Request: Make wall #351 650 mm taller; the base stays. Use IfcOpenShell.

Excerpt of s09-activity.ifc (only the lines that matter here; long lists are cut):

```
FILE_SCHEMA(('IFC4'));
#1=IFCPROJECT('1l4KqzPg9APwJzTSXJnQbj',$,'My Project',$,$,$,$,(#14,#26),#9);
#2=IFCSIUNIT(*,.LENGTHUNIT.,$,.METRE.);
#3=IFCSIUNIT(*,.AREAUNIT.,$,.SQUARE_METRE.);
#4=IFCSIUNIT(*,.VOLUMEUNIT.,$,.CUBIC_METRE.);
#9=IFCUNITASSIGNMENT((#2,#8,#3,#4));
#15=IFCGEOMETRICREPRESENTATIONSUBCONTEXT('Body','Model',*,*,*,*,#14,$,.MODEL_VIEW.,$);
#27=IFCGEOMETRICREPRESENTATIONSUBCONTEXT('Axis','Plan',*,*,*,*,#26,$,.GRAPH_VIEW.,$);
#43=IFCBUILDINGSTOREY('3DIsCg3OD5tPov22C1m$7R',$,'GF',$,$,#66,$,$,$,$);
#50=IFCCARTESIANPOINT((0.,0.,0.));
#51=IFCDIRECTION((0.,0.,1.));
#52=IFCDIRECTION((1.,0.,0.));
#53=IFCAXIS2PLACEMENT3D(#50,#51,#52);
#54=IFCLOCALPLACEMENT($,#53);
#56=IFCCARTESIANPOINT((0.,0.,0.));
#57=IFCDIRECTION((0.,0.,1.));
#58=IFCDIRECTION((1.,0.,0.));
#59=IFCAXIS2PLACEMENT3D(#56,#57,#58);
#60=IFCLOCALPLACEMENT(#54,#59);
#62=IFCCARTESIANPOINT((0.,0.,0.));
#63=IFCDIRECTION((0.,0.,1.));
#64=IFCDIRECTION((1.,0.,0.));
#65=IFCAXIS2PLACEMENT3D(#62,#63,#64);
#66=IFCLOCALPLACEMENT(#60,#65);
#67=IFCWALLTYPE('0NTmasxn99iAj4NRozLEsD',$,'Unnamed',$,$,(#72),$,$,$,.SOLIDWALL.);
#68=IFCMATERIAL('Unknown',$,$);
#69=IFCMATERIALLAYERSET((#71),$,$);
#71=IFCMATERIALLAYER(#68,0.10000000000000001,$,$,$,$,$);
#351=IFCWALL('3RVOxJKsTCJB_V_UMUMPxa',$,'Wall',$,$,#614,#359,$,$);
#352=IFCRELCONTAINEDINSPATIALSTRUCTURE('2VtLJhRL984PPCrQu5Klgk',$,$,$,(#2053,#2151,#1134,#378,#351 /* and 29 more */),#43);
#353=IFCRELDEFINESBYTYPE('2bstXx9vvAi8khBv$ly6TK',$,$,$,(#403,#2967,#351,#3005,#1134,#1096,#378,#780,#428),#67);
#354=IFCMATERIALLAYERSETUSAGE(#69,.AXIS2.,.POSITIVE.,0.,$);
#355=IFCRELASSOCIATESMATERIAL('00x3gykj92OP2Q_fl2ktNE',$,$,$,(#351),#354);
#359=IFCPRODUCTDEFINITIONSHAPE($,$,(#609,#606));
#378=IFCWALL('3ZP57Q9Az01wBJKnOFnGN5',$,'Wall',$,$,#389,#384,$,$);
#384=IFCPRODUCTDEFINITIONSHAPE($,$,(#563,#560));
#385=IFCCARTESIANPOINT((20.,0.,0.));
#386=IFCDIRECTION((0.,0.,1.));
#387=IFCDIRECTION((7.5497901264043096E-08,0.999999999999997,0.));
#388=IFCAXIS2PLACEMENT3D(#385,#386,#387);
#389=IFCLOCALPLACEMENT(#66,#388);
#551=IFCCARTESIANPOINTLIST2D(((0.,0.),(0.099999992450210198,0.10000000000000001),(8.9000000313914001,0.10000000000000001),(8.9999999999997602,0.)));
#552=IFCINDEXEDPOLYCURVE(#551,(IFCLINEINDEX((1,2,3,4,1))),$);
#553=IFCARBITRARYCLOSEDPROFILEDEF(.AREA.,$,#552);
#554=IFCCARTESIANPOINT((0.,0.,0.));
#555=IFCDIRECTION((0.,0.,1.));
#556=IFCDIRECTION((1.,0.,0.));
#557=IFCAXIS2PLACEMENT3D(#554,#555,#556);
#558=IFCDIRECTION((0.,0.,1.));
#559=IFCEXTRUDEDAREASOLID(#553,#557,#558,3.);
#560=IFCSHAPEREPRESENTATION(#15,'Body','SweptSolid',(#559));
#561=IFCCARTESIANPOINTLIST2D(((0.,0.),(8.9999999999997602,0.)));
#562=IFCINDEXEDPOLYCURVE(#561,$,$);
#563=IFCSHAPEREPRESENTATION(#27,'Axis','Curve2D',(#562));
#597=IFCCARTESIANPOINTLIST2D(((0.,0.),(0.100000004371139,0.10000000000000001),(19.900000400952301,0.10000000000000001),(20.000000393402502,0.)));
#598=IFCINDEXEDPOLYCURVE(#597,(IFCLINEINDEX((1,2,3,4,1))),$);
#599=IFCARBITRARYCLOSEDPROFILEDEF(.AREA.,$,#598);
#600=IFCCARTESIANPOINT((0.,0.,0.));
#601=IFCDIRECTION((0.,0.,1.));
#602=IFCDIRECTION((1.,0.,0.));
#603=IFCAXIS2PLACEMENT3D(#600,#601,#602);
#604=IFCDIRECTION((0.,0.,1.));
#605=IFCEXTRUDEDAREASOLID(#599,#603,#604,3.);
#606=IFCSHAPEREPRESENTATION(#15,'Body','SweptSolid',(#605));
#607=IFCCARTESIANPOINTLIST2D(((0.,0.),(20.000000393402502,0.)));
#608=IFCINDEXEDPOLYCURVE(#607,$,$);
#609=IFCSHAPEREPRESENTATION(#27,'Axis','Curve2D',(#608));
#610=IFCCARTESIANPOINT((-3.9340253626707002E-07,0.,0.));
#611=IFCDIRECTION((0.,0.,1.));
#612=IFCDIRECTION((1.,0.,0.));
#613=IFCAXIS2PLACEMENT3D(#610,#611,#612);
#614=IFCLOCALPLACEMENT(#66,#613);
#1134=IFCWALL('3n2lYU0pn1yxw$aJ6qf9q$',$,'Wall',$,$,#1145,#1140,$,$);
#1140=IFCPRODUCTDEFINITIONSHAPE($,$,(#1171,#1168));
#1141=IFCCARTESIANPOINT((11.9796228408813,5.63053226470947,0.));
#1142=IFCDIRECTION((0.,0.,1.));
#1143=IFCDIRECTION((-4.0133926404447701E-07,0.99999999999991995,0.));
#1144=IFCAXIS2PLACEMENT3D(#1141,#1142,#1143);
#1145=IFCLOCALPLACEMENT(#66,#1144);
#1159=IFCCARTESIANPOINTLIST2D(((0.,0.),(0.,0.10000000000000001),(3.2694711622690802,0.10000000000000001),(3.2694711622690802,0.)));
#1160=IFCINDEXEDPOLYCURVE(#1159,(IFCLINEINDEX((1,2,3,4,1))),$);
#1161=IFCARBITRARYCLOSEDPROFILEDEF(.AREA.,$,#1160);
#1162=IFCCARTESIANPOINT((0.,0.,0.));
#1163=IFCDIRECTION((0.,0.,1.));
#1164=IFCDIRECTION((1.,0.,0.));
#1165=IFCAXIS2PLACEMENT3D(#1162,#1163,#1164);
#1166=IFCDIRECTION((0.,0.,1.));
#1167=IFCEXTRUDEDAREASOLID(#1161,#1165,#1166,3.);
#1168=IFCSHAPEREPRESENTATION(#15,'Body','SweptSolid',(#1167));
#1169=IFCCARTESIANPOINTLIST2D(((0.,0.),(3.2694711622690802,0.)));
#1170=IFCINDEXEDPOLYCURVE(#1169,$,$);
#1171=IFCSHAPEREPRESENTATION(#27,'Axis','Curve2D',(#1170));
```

```python
import ifcopenshell
import ifcopenshell.geom
import ifcopenshell.util.representation
import ifcopenshell.util.shape

model = ifcopenshell.open("s09-activity.ifc")
settings = ifcopenshell.geom.settings()


def volume(element):
    """Net volume in cubic metres, openings subtracted."""
    shape = ifcopenshell.geom.create_shape(settings, element)
    return ifcopenshell.util.shape.get_volume(shape.geometry)


wall = model.by_guid("3RVOxJKsTCJB_V_UMUMPxa")
before = volume(wall)

body = ifcopenshell.util.representation.get_representation(wall, "Model", "Body")
solid = body.Items[0]
old_height = solid.Depth
solid.Depth += 0.65
after = volume(wall)

print(f"height {old_height:g} -> {solid.Depth:g}, volume {before:.3f} -> {after:.3f} m3")

model.write("s09-activity_updated.ifc")
```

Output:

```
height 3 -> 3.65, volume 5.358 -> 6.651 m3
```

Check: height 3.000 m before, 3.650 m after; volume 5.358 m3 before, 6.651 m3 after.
